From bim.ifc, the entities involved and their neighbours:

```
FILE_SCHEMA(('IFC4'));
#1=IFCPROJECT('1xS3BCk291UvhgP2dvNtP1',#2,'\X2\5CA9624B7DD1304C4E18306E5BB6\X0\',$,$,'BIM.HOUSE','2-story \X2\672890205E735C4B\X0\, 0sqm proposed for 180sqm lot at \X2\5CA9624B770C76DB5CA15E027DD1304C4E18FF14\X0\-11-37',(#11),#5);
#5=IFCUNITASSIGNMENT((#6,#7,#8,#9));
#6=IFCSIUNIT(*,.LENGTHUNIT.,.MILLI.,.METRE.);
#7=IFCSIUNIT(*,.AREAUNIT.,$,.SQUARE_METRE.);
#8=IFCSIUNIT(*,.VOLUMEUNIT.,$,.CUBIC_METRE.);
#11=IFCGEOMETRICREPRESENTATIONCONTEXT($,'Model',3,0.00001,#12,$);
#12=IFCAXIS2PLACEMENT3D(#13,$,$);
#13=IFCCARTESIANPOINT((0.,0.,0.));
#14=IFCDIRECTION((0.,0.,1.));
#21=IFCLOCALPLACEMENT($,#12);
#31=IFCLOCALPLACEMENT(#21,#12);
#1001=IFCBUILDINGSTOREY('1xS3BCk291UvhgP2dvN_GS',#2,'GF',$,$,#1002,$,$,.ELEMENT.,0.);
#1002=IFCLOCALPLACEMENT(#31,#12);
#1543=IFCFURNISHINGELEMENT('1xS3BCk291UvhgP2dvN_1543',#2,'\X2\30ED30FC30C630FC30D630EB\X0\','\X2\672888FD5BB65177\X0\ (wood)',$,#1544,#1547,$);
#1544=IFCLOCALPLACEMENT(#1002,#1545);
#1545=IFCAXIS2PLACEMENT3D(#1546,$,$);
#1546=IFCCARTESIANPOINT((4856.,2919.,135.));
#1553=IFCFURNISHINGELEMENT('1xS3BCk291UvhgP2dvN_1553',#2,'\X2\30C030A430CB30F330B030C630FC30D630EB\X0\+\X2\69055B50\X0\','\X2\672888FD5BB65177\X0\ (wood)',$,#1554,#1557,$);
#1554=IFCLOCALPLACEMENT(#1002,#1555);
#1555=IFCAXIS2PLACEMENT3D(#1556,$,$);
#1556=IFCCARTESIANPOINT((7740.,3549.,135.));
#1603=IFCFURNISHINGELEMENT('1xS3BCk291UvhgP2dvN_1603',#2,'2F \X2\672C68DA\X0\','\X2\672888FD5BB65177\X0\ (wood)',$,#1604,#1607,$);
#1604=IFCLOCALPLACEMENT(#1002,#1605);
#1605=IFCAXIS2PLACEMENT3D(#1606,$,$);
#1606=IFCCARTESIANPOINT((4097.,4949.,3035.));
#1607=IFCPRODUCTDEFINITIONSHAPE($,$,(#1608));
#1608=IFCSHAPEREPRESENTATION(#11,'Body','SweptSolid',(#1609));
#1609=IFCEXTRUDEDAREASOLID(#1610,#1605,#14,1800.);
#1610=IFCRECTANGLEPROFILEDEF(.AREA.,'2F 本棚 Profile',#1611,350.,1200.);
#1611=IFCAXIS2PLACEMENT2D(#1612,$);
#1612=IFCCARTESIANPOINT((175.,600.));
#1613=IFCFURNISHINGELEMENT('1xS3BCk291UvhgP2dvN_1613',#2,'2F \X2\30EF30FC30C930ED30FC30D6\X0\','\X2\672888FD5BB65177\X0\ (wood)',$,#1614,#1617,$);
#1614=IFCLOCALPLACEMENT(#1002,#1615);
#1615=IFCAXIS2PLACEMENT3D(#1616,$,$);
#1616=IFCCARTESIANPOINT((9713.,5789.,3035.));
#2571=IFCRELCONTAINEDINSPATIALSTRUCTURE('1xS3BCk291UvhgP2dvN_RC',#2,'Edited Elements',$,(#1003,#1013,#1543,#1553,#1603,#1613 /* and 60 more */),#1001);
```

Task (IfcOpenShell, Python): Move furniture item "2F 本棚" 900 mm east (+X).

```python
import ifcopenshell
import ifcopenshell.api.geometry
import ifcopenshell.util.placement
import ifcopenshell.util.unit

model = ifcopenshell.open("bim.ifc")
unit_scale = ifcopenshell.util.unit.calculate_unit_scale(model)

item = model.by_guid("1xS3BCk291UvhgP2dvN_1603")
matrix = ifcopenshell.util.placement.get_local_placement(item.ObjectPlacement)
matrix[0, 3] += 0.9 / unit_scale
ifcopenshell.api.geometry.edit_object_placement(model, product=item, matrix=matrix, is_si=False)

print(ifcopenshell.util.placement.get_local_placement(item.ObjectPlacement).round(3) + 0.0)

model.write("bim-out.ifc")
```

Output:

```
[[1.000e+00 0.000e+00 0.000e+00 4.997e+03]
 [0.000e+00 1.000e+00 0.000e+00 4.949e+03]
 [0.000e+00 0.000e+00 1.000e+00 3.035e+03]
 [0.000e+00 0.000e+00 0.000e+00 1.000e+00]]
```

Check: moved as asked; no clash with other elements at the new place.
